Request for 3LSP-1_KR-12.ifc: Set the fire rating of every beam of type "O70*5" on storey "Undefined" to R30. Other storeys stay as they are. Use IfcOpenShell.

First a look at what the model holds.

```python
import ifcopenshell
import ifcopenshell.util.element

model = ifcopenshell.open("3LSP-1_KR-12.ifc")
print(model.schema)
storey = next(s for s in model.by_type("IfcBuildingStorey") if s.Name == "Undefined")
beams = [e for e in ifcopenshell.util.element.get_decomposition(storey) if e.is_a("IfcBeam")]
seen = {}
for e in beams:
    element_type = ifcopenshell.util.element.get_type(e)
    key = (element_type.Name if element_type != e and element_type else None, ifcopenshell.util.element.get_pset(e, "Pset_BeamCommon", "FireRating"))
    seen[key] = seen.get(key, 0) + 1
for (name, value), count in sorted(seen.items(), key=str):
    print(count, "x", name, "|", value)
```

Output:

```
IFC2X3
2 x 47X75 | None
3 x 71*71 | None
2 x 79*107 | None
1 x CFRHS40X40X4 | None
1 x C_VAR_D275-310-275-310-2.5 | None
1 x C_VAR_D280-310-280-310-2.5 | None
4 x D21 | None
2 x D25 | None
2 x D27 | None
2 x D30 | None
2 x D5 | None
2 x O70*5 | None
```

```python
import ifcopenshell
import ifcopenshell.api.pset
import ifcopenshell.util.element

model = ifcopenshell.open("3LSP-1_KR-12.ifc")

storey = next(s for s in model.by_type("IfcBuildingStorey") if s.Name == "Undefined")
beams = [e for e in ifcopenshell.util.element.get_decomposition(storey) if e.is_a("IfcBeam")]

count = 0
for e in beams:
    element_type = ifcopenshell.util.element.get_type(e)
    if element_type in (None, e) or element_type.Name != "O70*5":
        continue
    found = ifcopenshell.util.element.get_pset(e, "Pset_BeamCommon", should_inherit=False)
    if found:
        pset = model.by_id(found["id"])
        if len(ifcopenshell.util.element.get_elements_by_pset(pset)) > 1:
            pset = ifcopenshell.api.pset.unshare_pset(model, products=[e], pset=pset)[0]
    else:
        pset = ifcopenshell.api.pset.add_pset(model, product=e, name="Pset_BeamCommon")
    ifcopenshell.api.pset.edit_pset(model, pset=pset, properties={"FireRating": "R30"})
    count += 1

print(count, "beams updated")

model.write("3LSP-1_KR-12_v2.ifc")
```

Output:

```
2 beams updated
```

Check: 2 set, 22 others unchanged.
